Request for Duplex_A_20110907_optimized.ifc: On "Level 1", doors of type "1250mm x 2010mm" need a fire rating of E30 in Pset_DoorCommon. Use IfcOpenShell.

First a look at what the model holds.

```python
import ifcopenshell
import ifcopenshell.util.element

model = ifcopenshell.open("Duplex_A_20110907_optimized.ifc")
print(model.schema)
storey = next(s for s in model.by_type("IfcBuildingStorey") if s.Name == "Level 1")
doors = [e for e in ifcopenshell.util.element.get_decomposition(storey) if e.is_a("IfcDoor")]
seen = {}
for e in doors:
    element_type = ifcopenshell.util.element.get_type(e)
    key = (element_type.Name if element_type != e and element_type else None, ifcopenshell.util.element.get_pset(e, "Pset_DoorCommon", "FireRating"))
    seen[key] = seen.get(key, 0) + 1
for (name, value), count in sorted(seen.items(), key=str):
    print(count, "x", name, "|", value)
```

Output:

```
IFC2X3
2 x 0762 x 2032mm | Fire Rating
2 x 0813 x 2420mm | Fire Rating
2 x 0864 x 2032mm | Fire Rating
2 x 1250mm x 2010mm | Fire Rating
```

```python
import ifcopenshell
import ifcopenshell.api.pset
import ifcopenshell.util.element

model = ifcopenshell.open("Duplex_A_20110907_optimized.ifc")

storey = next(s for s in model.by_type("IfcBuildingStorey") if s.Name == "Level 1")
doors = [e for e in ifcopenshell.util.element.get_decomposition(storey) if e.is_a("IfcDoor")]

count = 0
for e in doors:
    element_type = ifcopenshell.util.element.get_type(e)
    if element_type in (None, e) or element_type.Name != "1250mm x 2010mm":
        continue
    # add_pset returns the element's existing set when there is one.
    pset = ifcopenshell.api.pset.add_pset(model, product=e, name="Pset_DoorCommon")
    ifcopenshell.api.pset.edit_pset(model, pset=pset, properties={"FireRating": "E30"})
    count += 1

print(count, "doors updated")

model.write("Duplex_A_20110907_optimized_edited.ifc")
```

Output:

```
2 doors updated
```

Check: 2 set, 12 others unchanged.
